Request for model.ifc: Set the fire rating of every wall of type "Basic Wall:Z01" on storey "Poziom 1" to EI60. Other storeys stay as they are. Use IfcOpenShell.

First a look at what the model holds.

```python
import ifcopenshell
import ifcopenshell.util.element

model = ifcopenshell.open("model.ifc")
print(model.schema)
storey = next(s for s in model.by_type("IfcBuildingStorey") if s.Name == "Poziom 1")
walls = [e for e in ifcopenshell.util.element.get_decomposition(storey) if e.is_a("IfcWall")]
seen = {}
for e in walls:
    element_type = ifcopenshell.util.element.get_type(e)
    key = (element_type.Name if element_type != e and element_type else None, ifcopenshell.util.element.get_pset(e, "Pset_WallCommon", "FireRating"))
    seen[key] = seen.get(key, 0) + 1
for (name, value), count in sorted(seen.items(), key=str):
    print(count, "x", name, "|", value)
```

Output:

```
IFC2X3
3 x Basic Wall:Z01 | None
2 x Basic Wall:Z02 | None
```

```python
import ifcopenshell
import ifcopenshell.api.pset
import ifcopenshell.util.element

model = ifcopenshell.open("model.ifc")

storey = next(s for s in model.by_type("IfcBuildingStorey") if s.Name == "Poziom 1")
walls = [e for e in ifcopenshell.util.element.get_decomposition(storey) if e.is_a("IfcWall")]

count = 0
for e in walls:
    element_type = ifcopenshell.util.element.get_type(e)
    if element_type in (None, e) or element_type.Name != "Basic Wall:Z01":
        continue
    found = ifcopenshell.util.element.get_pset(e, "Pset_WallCommon", should_inherit=False)
    if found:
        pset = model.by_id(found["id"])
        if len(ifcopenshell.util.element.get_elements_by_pset(pset)) > 1:
            pset = ifcopenshell.api.pset.unshare_pset(model, products=[e], pset=pset)[0]
    else:
        pset = ifcopenshell.api.pset.add_pset(model, product=e, name="Pset_WallCommon")
    ifcopenshell.api.pset.edit_pset(model, pset=pset, properties={"FireRating": "EI60"})
    count += 1

print(count, "walls updated")

model.write("model_edited.ifc")
```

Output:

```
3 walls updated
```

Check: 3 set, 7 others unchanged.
